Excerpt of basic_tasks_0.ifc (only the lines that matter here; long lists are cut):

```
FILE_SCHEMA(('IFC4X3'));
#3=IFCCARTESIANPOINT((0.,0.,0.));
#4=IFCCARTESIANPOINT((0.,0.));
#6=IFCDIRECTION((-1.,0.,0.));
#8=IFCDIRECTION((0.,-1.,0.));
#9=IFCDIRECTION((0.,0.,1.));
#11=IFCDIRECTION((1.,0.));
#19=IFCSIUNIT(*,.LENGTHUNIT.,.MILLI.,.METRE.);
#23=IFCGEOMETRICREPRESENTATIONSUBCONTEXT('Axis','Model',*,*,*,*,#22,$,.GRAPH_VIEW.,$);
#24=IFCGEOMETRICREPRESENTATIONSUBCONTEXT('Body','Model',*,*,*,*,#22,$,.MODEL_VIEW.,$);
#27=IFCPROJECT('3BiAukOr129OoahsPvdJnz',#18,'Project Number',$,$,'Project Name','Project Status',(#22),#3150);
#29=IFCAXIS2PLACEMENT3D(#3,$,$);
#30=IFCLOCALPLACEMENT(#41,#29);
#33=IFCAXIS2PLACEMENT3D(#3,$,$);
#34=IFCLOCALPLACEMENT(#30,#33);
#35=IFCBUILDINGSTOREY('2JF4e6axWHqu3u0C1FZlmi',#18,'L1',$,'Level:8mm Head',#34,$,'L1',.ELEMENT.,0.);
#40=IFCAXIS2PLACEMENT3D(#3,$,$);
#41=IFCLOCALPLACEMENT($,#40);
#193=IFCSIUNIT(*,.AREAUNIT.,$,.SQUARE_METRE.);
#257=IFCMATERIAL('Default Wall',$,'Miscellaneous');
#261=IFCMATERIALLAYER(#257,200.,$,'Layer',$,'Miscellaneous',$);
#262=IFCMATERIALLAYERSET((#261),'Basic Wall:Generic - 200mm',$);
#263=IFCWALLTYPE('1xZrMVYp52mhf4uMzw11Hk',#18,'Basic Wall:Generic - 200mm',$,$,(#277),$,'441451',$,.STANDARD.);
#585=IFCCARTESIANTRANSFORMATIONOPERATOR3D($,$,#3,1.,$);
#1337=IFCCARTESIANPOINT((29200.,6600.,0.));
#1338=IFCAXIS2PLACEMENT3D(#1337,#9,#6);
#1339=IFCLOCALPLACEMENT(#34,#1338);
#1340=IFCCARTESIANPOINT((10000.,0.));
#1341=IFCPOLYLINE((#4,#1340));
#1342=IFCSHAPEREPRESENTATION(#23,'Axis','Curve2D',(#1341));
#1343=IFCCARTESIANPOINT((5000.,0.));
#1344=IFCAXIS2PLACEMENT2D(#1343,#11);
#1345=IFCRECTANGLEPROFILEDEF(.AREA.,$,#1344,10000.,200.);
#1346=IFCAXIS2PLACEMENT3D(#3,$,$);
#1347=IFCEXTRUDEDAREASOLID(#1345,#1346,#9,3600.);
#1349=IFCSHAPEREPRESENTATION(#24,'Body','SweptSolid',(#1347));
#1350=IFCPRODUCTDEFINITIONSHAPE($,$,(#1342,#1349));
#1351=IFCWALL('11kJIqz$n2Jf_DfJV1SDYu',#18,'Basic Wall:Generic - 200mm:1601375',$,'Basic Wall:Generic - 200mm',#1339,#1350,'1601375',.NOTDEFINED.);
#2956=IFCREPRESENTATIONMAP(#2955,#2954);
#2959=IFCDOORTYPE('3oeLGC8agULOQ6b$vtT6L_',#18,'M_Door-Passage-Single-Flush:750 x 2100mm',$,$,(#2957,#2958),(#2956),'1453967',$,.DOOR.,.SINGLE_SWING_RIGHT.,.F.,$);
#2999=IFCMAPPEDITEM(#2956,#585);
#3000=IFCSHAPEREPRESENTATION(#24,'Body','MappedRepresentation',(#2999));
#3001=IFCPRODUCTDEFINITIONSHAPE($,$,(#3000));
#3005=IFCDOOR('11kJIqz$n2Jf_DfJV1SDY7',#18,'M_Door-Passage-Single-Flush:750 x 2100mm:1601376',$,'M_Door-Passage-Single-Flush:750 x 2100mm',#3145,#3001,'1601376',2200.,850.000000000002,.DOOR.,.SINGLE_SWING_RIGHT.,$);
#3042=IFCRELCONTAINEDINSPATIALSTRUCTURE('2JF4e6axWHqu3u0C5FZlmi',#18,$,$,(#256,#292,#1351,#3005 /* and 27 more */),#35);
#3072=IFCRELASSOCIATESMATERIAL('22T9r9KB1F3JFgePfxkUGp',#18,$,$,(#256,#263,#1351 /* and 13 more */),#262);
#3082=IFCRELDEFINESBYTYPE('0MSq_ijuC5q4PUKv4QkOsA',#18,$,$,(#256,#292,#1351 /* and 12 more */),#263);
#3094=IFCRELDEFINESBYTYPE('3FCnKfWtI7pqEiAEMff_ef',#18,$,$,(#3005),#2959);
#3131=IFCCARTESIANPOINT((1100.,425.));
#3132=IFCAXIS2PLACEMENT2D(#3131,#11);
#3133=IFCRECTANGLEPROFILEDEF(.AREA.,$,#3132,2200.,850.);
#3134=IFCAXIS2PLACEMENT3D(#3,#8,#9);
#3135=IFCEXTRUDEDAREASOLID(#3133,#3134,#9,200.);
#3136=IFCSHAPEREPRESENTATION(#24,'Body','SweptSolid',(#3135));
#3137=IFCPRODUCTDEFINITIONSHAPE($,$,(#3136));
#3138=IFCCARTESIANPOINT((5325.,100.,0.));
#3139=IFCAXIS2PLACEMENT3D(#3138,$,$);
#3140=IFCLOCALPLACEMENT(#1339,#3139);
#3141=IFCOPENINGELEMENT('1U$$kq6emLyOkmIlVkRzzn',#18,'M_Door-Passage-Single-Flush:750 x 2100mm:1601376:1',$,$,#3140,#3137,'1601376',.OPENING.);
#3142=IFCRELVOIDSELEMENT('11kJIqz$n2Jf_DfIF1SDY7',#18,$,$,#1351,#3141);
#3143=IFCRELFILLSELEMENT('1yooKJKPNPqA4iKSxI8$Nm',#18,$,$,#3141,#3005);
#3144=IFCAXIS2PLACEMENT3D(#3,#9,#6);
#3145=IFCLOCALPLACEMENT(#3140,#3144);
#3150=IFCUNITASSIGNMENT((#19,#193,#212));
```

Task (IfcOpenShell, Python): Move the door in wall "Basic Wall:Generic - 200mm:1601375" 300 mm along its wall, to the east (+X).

```python
import ifcopenshell
import ifcopenshell.api.geometry
import ifcopenshell.util.placement

model = ifcopenshell.open("basic_tasks_0.ifc")

door = model.by_guid("11kJIqz$n2Jf_DfJV1SDY7")
opening = door.FillsVoids[0].RelatingOpeningElement
wall = opening.VoidsElements[0].RelatingBuildingElement

wall_matrix = ifcopenshell.util.placement.get_local_placement(wall.ObjectPlacement)
shift = wall_matrix[:3, 0] * -300.0
before = ifcopenshell.util.placement.get_local_placement(door.ObjectPlacement)[:3, 3].copy()

# The door is placed relative to its opening, so it follows when the opening moves.
matrix = ifcopenshell.util.placement.get_local_placement(opening.ObjectPlacement)
matrix[:3, 3] += shift
ifcopenshell.api.geometry.edit_object_placement(
    model, product=opening, matrix=matrix, is_si=False, should_transform_children=True
)

after = ifcopenshell.util.placement.get_local_placement(door.ObjectPlacement)[:3, 3]
print("door moved by", (after - before).round(3) + 0.0)

model.write("basic_tasks_0_v2.ifc")
```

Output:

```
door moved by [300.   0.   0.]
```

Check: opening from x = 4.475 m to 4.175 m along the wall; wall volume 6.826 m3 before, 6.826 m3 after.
